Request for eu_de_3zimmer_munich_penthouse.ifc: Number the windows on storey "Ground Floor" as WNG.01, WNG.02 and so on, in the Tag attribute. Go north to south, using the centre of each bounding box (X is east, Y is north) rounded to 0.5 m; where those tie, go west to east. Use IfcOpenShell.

First a look at what the model holds.

```python
import ifcopenshell
import ifcopenshell.util.element
import ifcopenshell.util.placement

model = ifcopenshell.open("eu_de_3zimmer_munich_penthouse.ifc")
print(model.schema)
storey = next(s for s in model.by_type("IfcBuildingStorey") if s.Name == "Ground Floor")
windows = [e for e in ifcopenshell.util.element.get_decomposition(storey) if e.is_a("IfcWindow")]
for e in sorted(windows, key=lambda e: e.id()):
    origin = ifcopenshell.util.placement.get_local_placement(e.ObjectPlacement)[:3, 3]
    print(e.id(), e.Tag, e.Name, origin.round(2) + 0.0, sep=" | ")
```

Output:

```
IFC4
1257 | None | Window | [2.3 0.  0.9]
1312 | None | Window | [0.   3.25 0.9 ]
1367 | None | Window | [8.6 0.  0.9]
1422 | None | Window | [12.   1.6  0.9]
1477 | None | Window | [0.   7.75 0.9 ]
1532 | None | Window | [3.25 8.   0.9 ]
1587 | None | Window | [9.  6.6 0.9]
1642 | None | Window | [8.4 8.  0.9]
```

```python
import ifcopenshell
import ifcopenshell.geom
import ifcopenshell.util.element
import ifcopenshell.util.shape

model = ifcopenshell.open("eu_de_3zimmer_munich_penthouse.ifc")
settings = ifcopenshell.geom.settings()
settings.set("use-world-coords", True)


def centre(element):
    shape = ifcopenshell.geom.create_shape(settings, element)
    return ifcopenshell.util.shape.get_bbox_centroid(shape.geometry)


storey = next(s for s in model.by_type("IfcBuildingStorey") if s.Name == "Ground Floor")
windows = [e for e in ifcopenshell.util.element.get_decomposition(storey) if e.is_a("IfcWindow")]

# Insertion points can sit at a corner or the storey origin, so sort by the geometry (in metres).
centres = {e: centre(e) for e in windows}
windows.sort(key=lambda e: (-round(centres[e][1] / 0.5), centres[e][0]))

for i, e in enumerate(windows, start=1):
    number = f"WNG.{i:02d}"
    e.Tag = number
    print(e.id(), number)

model.write("eu_de_3zimmer_munich_penthouse-out.ifc")
```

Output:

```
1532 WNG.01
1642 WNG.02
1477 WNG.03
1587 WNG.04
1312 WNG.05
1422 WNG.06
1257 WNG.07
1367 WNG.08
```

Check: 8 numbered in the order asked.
